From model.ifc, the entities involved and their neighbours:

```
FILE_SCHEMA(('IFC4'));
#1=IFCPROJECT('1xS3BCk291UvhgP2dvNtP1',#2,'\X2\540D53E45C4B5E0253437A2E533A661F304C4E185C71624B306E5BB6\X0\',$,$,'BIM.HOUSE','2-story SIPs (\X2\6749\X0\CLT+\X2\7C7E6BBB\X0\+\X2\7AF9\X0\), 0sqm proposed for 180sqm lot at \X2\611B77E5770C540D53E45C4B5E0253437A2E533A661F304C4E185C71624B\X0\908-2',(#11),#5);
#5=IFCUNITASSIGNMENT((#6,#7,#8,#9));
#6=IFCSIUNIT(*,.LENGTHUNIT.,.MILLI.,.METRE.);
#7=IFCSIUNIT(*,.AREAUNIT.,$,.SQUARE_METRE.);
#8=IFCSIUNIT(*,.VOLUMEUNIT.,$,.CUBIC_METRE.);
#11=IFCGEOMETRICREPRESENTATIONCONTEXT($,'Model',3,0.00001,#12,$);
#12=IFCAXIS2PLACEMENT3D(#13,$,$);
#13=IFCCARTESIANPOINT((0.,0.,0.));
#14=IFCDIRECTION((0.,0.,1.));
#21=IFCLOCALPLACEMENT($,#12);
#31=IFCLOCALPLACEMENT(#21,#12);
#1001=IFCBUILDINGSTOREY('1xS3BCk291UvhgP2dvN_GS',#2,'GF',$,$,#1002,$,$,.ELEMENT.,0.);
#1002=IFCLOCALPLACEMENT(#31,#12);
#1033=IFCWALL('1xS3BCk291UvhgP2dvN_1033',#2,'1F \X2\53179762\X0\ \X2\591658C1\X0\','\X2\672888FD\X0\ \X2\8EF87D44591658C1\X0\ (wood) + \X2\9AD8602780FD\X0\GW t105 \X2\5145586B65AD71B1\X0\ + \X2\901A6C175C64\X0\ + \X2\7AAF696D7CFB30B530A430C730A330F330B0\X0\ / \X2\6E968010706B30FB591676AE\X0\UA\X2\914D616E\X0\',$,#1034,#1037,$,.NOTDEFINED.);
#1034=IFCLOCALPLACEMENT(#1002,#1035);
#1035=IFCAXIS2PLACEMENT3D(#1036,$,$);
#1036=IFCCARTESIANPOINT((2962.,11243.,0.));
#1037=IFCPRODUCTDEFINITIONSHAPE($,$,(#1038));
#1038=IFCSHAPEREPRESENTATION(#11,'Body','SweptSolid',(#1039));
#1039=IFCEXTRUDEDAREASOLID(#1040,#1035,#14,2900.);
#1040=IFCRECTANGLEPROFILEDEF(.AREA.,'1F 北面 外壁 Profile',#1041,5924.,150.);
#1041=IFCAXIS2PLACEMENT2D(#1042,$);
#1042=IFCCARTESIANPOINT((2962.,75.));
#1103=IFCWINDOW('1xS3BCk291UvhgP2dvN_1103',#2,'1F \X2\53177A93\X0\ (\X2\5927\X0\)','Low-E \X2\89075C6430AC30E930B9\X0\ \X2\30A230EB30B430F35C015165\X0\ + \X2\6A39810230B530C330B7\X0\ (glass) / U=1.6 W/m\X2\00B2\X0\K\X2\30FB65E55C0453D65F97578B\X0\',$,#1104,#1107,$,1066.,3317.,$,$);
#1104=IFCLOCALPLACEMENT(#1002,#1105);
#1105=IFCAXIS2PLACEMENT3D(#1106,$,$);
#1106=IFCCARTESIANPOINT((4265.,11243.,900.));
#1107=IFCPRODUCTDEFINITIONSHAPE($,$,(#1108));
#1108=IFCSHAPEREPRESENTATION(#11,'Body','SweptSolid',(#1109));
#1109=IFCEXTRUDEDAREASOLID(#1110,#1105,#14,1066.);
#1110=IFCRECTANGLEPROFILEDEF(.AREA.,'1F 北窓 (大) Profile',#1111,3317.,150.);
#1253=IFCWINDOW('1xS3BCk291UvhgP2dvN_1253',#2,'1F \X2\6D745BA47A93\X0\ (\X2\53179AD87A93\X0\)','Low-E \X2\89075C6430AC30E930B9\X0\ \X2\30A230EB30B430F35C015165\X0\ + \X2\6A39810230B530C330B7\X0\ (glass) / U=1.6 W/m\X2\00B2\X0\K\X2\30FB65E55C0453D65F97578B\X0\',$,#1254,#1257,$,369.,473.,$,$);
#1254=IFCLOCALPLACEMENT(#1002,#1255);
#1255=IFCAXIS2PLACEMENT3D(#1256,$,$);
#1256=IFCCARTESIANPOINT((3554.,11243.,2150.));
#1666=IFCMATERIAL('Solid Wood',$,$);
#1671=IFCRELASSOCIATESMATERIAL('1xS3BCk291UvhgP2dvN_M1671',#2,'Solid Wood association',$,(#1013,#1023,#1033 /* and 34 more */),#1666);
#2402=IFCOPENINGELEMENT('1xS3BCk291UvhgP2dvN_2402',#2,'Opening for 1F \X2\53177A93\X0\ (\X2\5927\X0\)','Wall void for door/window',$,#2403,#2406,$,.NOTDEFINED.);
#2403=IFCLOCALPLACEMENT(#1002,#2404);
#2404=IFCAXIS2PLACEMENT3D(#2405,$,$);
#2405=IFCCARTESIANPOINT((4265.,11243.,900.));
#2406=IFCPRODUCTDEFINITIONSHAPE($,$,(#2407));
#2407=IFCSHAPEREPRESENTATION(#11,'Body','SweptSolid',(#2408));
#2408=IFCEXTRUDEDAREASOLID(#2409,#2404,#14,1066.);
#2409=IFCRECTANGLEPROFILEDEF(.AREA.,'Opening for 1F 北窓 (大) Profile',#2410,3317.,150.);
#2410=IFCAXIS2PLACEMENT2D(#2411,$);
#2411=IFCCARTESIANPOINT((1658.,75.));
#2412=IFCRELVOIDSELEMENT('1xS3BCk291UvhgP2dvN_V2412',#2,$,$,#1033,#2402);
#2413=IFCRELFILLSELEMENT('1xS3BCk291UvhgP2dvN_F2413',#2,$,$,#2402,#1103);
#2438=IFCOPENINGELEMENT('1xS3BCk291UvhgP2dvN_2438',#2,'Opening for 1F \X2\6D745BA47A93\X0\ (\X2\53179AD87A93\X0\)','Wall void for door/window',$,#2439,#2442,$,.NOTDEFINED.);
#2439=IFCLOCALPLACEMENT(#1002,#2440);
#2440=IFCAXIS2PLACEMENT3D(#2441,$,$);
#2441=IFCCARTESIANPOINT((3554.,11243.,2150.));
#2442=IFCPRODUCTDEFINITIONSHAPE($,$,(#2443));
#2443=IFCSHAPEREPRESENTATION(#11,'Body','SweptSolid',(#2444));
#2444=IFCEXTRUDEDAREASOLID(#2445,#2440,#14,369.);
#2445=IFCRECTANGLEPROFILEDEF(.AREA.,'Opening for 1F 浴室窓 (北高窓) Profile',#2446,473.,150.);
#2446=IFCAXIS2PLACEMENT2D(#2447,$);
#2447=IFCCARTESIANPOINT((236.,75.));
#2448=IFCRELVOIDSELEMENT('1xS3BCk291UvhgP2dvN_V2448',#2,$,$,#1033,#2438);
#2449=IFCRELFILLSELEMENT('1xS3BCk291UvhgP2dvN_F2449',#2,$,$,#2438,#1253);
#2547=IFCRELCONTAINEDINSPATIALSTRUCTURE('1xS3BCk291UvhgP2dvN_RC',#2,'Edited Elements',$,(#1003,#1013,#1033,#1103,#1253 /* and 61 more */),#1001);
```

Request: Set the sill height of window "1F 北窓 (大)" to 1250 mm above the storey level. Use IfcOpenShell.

```python
import numpy as np
import ifcopenshell
import ifcopenshell.api.geometry
import ifcopenshell.geom
import ifcopenshell.util.element
import ifcopenshell.util.placement
import ifcopenshell.util.shape
import ifcopenshell.util.unit

model = ifcopenshell.open("model.ifc")
unit_scale = ifcopenshell.util.unit.calculate_unit_scale(model)

window = model.by_guid("1xS3BCk291UvhgP2dvN_1103")
opening = window.FillsVoids[0].RelatingOpeningElement
storey = ifcopenshell.util.element.get_container(window, ifc_class="IfcBuildingStorey")
level = ifcopenshell.util.placement.get_local_placement(storey.ObjectPlacement)[2, 3]

# The opening's origin need not be at the sill, so measure its lowest point.
shape = ifcopenshell.geom.create_shape(ifcopenshell.geom.settings(), opening)
bottom = ifcopenshell.util.shape.get_shape_bottom_elevation(shape, shape.geometry) / unit_scale
dz = level + 1.25 / unit_scale - bottom

shift = np.array([0.0, 0.0, dz])
# The window is not placed relative to its opening, so move both.
for product in (opening, window):
    matrix = ifcopenshell.util.placement.get_local_placement(product.ObjectPlacement)
    matrix[:3, 3] += shift
    ifcopenshell.api.geometry.edit_object_placement(model, product=product, matrix=matrix, is_si=False)

print(f"moved by {dz * unit_scale:+.3f} m")

model.write("model_rev.ifc")
```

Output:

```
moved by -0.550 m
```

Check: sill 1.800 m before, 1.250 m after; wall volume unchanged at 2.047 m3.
